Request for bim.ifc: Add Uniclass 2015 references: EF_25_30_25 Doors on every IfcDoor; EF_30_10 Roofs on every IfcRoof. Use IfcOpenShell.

First a look at what the model holds.

```python
import ifcopenshell

model = ifcopenshell.open("bim.ifc")
print(model.schema)
print("classifications:", [c.Name for c in model.by_type("IfcClassification")])
for ifc_class in ("IfcDoor", "IfcRoof", "IfcStair", "IfcWall", "IfcWindow"):
    print(ifc_class, len(model.by_type(ifc_class)))
```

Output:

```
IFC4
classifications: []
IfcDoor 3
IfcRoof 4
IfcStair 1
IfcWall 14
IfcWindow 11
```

```python
import ifcopenshell
import ifcopenshell.api.classification

model = ifcopenshell.open("bim.ifc")

system = ifcopenshell.api.classification.add_classification(model, classification="Uniclass 2015")

codes = {
    "IfcDoor": ("EF_25_30_25", "Doors"),
    "IfcRoof": ("EF_30_10", "Roofs"),
}
for ifc_class, (code, name) in codes.items():
    products = model.by_type(ifc_class)
    ifcopenshell.api.classification.add_reference(
        model, products=products, classification=system, identification=code, name=name
    )
    print(code, len(products))

model.write("bim_v2.ifc")
```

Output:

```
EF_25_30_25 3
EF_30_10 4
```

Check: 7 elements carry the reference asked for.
